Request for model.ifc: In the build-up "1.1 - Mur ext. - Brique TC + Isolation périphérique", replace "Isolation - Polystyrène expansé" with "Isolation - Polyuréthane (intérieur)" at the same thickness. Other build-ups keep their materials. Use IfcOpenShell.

First a look at what the model holds.

```python
import ifcopenshell
import ifcopenshell.util.element

model = ifcopenshell.open("model.ifc")
print(model.schema)
for layer_set in model.by_type("IfcMaterialLayerSet"):
    if layer_set.LayerSetName == "1.1 - Mur ext. - Brique TC + Isolation périphérique":
        for layer in layer_set.MaterialLayers:
            print(layer.id(), layer.Material and layer.Material.Name, layer.LayerThickness, sep=" | ")
        print(len(ifcopenshell.util.element.get_elements_by_material(model, layer_set)), "elements and types use it")
print(sorted(m.Name for m in model.by_type("IfcMaterial") if m.Name)[:60])
```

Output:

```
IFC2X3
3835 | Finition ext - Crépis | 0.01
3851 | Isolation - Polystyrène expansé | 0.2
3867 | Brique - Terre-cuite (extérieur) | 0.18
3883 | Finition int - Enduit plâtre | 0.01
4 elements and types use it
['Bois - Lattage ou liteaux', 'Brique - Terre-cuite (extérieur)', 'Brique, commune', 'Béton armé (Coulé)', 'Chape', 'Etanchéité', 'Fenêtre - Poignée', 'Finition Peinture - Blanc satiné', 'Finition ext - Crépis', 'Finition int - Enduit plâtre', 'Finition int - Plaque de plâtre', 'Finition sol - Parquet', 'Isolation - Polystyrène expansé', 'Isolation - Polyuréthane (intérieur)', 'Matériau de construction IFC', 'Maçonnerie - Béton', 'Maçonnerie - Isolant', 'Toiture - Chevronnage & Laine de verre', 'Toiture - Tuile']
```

```python
import ifcopenshell
import ifcopenshell.api.material

model = ifcopenshell.open("model.ifc")

layer_set = next(s for s in model.by_type("IfcMaterialLayerSet") if s.LayerSetName == "1.1 - Mur ext. - Brique TC + Isolation périphérique")
layer = next(l for l in layer_set.MaterialLayers if l.Material and l.Material.Name == "Isolation - Polystyrène expansé")
material = next(m for m in model.by_type("IfcMaterial") if m.Name == "Isolation - Polyuréthane (intérieur)")

# Point this one layer at the other material; renaming the old one would change it everywhere.
ifcopenshell.api.material.edit_layer(model, layer=layer, attributes={}, material=material)

print([l.Material.Name if l.Material else None for l in layer_set.MaterialLayers])

model.write("model_edited.ifc")
```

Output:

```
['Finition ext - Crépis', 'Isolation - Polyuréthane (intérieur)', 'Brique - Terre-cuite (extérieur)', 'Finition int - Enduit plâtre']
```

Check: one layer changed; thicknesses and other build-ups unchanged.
